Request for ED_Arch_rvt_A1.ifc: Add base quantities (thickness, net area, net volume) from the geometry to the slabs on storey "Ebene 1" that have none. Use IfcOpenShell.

First a look at what the model holds.

```python
import ifcopenshell
import ifcopenshell.util.element
import ifcopenshell.util.unit

model = ifcopenshell.open("ED_Arch_rvt_A1.ifc")
print(model.schema)
for unit_type in ("LENGTHUNIT", "AREAUNIT", "VOLUMEUNIT"):
    print(unit_type, ifcopenshell.util.unit.calculate_unit_scale(model, unit_type))
storey = next(s for s in model.by_type("IfcBuildingStorey") if s.Name == "Ebene 1")
slabs = [e for e in ifcopenshell.util.element.get_decomposition(storey) if e.is_a("IfcSlab")]
for e in sorted(slabs, key=lambda e: e.id()):
    print(e.id(), e.is_a(), e.Name, list(ifcopenshell.util.element.get_psets(e, qtos_only=True)), sep=" | ")
```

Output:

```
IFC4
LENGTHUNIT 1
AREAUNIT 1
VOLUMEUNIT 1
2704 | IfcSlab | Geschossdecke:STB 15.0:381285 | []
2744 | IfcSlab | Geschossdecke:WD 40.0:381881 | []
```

```python
import ifcopenshell
import ifcopenshell.api.pset
import ifcopenshell.geom
import ifcopenshell.util.element
import ifcopenshell.util.shape
import ifcopenshell.util.unit

model = ifcopenshell.open("ED_Arch_rvt_A1.ifc")
unit_scale = ifcopenshell.util.unit.calculate_unit_scale(model)
area_scale = ifcopenshell.util.unit.calculate_unit_scale(model, "AREAUNIT")
volume_scale = ifcopenshell.util.unit.calculate_unit_scale(model, "VOLUMEUNIT")
settings = ifcopenshell.geom.settings()

storey = next(s for s in model.by_type("IfcBuildingStorey") if s.Name == "Ebene 1")
slabs = [e for e in ifcopenshell.util.element.get_decomposition(storey) if e.is_a("IfcSlab")]

for e in sorted(slabs, key=lambda e: e.id()):
    if ifcopenshell.util.element.get_psets(e, qtos_only=True, should_inherit=False):
        continue
    # Geometry comes back in metres, in the element's own axes.
    shape = ifcopenshell.geom.create_shape(settings, e)
    values = {
        "Width": ifcopenshell.util.shape.get_z(shape.geometry) / unit_scale,
        "NetArea": ifcopenshell.util.shape.get_footprint_area(shape.geometry) / area_scale,
        "NetVolume": ifcopenshell.util.shape.get_volume(shape.geometry) / volume_scale,
    }
    qto = ifcopenshell.api.pset.add_qto(model, product=e, name="Qto_SlabBaseQuantities")
    ifcopenshell.api.pset.edit_qto(model, qto=qto, properties=values)
    print(e.id(), {k: round(v, 3) for k, v in values.items()})

model.write("ED_Arch_rvt_A1_v2.ifc")
```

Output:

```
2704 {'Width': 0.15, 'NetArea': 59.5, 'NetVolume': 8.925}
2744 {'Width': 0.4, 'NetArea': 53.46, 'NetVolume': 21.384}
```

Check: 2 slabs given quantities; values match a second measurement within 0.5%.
